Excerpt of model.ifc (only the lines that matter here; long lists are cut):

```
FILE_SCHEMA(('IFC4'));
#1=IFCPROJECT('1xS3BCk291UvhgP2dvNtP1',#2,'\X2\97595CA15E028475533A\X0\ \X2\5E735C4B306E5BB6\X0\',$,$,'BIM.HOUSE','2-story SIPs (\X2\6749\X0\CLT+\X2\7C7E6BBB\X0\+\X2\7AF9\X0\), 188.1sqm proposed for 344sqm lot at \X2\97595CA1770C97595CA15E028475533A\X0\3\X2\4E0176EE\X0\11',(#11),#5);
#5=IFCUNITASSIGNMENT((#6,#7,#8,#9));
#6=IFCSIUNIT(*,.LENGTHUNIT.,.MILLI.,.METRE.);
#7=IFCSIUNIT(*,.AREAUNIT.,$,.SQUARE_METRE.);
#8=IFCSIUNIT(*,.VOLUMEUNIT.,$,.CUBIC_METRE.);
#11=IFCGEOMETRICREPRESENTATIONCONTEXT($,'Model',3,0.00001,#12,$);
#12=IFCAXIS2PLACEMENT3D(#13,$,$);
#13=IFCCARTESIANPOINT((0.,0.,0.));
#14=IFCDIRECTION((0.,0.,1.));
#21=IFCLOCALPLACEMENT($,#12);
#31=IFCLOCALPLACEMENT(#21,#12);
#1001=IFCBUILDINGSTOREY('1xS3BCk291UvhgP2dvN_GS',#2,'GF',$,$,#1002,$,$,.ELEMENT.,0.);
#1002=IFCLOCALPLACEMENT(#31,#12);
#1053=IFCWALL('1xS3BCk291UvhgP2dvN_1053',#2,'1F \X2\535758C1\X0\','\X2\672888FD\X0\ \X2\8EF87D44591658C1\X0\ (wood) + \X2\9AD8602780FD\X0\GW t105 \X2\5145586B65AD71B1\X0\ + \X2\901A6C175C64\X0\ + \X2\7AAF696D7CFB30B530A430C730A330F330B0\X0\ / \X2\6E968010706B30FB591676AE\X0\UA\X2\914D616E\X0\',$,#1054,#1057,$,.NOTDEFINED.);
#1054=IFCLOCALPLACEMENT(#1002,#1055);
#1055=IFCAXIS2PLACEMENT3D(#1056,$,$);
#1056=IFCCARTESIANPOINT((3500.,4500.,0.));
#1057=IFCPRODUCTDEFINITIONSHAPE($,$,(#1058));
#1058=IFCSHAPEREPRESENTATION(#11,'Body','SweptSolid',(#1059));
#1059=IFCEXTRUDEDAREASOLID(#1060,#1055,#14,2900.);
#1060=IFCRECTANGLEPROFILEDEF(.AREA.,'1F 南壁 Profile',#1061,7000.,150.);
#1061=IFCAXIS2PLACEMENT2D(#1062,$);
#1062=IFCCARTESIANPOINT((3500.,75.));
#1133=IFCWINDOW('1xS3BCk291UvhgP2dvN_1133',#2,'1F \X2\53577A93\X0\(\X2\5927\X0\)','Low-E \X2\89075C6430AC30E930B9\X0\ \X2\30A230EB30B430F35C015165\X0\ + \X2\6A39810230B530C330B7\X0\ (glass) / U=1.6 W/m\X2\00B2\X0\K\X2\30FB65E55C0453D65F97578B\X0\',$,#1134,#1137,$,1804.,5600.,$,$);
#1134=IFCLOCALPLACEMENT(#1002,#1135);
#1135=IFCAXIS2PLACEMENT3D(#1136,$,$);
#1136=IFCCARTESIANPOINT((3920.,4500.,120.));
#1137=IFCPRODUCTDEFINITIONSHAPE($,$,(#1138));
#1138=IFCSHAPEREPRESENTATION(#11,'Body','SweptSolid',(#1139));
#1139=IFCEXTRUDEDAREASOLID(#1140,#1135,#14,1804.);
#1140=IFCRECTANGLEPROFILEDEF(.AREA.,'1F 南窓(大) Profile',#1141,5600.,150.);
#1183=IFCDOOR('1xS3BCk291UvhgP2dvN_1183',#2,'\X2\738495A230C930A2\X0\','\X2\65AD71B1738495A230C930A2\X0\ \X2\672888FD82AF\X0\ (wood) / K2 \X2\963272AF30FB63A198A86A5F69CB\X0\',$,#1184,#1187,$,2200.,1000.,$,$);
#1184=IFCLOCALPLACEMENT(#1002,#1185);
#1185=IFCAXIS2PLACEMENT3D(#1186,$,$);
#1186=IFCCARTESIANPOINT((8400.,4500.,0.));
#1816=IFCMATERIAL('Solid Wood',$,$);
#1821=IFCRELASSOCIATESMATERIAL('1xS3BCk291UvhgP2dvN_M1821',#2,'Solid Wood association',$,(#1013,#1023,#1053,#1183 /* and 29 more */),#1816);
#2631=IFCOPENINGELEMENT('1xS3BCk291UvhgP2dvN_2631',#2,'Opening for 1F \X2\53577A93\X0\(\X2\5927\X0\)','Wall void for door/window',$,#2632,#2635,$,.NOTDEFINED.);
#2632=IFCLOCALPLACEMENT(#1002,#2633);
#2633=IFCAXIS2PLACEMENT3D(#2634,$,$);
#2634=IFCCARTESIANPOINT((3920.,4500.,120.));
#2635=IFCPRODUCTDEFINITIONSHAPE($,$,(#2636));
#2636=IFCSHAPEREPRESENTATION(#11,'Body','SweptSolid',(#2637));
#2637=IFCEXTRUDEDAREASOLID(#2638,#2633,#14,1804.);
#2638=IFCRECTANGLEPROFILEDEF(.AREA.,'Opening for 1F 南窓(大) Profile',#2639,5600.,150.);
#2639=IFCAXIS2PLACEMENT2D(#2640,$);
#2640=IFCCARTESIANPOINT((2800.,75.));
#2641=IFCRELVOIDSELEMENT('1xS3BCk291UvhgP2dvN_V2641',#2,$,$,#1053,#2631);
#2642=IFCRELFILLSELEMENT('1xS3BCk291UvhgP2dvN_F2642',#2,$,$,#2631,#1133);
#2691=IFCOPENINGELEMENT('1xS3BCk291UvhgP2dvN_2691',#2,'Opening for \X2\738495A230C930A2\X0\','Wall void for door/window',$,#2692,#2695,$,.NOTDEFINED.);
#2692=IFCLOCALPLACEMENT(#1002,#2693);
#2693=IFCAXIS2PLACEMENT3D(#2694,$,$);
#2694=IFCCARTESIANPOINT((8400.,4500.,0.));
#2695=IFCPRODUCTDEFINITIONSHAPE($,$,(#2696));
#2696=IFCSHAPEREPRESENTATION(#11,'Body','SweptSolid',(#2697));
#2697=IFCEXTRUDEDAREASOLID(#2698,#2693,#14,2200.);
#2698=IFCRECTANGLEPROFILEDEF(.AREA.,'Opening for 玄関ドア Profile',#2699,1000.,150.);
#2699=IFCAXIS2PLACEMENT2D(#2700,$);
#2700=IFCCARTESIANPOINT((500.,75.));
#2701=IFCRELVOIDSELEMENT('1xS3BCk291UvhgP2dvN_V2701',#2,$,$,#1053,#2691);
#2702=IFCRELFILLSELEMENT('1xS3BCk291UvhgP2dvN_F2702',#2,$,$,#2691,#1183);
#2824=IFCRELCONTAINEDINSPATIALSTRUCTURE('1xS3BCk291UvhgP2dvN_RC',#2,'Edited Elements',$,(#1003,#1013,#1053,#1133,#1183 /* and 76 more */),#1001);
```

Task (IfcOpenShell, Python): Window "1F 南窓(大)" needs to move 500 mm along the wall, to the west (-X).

```python
import ifcopenshell
import ifcopenshell.api.geometry
import ifcopenshell.util.placement
import ifcopenshell.util.unit

model = ifcopenshell.open("model.ifc")
unit_scale = ifcopenshell.util.unit.calculate_unit_scale(model)

window = model.by_id(1133)
opening = window.FillsVoids[0].RelatingOpeningElement
wall = opening.VoidsElements[0].RelatingBuildingElement

wall_matrix = ifcopenshell.util.placement.get_local_placement(wall.ObjectPlacement)
shift = wall_matrix[:3, 0] * -0.5 / unit_scale
before = ifcopenshell.util.placement.get_local_placement(window.ObjectPlacement)[:3, 3].copy()

# The window is not placed relative to its opening, so move both.
for product in (opening, window):
    matrix = ifcopenshell.util.placement.get_local_placement(product.ObjectPlacement)
    matrix[:3, 3] += shift
    ifcopenshell.api.geometry.edit_object_placement(model, product=product, matrix=matrix, is_si=False)

after = ifcopenshell.util.placement.get_local_placement(window.ObjectPlacement)[:3, 3]
print("window moved by", (after - before).round(3) + 0.0)

model.write("model_updated.ifc")
```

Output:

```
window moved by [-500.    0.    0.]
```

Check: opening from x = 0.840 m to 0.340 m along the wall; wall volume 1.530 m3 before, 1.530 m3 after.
